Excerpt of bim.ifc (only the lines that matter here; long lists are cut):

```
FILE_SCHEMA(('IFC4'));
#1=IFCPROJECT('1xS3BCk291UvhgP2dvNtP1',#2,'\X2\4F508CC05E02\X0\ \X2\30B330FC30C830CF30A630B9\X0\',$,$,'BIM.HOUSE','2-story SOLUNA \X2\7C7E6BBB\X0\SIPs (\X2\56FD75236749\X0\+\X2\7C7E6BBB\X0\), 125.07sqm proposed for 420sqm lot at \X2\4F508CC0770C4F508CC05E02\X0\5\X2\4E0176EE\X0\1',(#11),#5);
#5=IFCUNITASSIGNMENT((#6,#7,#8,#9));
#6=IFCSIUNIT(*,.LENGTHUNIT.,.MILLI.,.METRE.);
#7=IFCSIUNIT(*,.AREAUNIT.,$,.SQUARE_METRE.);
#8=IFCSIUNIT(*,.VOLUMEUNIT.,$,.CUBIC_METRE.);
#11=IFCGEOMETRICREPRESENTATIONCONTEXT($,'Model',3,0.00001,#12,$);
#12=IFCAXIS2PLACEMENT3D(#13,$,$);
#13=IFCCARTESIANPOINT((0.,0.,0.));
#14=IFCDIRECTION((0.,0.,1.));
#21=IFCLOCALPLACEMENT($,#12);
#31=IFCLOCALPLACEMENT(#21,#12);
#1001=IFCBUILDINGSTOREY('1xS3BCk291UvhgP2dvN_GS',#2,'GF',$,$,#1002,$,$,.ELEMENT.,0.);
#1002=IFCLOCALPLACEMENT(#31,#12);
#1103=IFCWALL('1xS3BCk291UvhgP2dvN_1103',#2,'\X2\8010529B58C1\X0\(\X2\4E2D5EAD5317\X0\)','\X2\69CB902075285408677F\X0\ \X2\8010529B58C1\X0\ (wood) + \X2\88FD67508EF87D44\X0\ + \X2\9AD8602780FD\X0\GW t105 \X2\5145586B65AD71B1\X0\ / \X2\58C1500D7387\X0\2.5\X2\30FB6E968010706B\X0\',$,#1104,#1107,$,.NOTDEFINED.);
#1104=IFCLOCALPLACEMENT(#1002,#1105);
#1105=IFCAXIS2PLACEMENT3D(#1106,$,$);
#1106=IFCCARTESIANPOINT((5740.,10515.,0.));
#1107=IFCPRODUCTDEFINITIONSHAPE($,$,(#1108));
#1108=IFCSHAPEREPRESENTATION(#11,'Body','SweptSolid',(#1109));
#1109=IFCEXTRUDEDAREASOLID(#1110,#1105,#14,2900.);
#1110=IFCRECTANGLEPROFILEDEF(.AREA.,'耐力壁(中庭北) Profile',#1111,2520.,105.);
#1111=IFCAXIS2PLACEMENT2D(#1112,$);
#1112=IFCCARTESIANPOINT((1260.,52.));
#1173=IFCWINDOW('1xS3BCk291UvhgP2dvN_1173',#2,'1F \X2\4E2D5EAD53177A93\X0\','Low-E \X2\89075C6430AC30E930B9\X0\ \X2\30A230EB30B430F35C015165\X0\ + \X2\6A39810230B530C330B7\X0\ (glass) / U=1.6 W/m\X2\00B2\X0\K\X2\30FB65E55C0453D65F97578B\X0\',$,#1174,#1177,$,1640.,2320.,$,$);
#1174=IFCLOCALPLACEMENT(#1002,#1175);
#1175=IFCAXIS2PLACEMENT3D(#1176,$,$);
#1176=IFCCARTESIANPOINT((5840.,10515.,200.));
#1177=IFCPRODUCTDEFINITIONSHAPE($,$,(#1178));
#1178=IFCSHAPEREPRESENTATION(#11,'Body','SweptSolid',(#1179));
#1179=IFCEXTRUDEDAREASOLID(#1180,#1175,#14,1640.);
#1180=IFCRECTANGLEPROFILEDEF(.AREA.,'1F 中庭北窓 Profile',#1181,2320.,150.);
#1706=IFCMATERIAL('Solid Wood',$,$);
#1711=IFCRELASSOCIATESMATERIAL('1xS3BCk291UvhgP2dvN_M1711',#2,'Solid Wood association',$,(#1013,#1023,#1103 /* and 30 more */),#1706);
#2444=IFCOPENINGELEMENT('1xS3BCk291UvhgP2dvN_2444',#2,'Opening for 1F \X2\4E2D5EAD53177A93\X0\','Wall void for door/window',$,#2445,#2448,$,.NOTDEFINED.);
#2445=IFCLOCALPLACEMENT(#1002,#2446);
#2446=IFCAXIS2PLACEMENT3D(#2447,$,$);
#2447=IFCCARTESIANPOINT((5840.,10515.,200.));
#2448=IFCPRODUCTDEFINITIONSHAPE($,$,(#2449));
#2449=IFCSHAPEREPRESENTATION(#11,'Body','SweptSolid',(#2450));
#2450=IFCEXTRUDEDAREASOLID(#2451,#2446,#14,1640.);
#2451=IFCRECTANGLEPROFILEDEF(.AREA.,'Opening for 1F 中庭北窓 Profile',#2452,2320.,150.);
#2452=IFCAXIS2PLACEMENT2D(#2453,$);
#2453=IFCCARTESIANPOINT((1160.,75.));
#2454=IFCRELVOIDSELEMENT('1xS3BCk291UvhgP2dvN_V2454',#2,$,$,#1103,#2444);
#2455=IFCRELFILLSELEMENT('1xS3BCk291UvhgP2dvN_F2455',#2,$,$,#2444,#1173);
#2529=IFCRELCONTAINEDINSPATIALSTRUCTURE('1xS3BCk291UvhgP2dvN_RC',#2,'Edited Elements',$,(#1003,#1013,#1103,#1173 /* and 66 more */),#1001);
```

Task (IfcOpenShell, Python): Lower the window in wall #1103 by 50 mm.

```python
import numpy as np
import ifcopenshell
import ifcopenshell.api.geometry
import ifcopenshell.util.placement
import ifcopenshell.util.unit

model = ifcopenshell.open("bim.ifc")
unit_scale = ifcopenshell.util.unit.calculate_unit_scale(model)

window = model.by_id(1173)
opening = window.FillsVoids[0].RelatingOpeningElement
dz = -0.05 / unit_scale

shift = np.array([0.0, 0.0, dz])
# The window is not placed relative to its opening, so move both.
for product in (opening, window):
    matrix = ifcopenshell.util.placement.get_local_placement(product.ObjectPlacement)
    matrix[:3, 3] += shift
    ifcopenshell.api.geometry.edit_object_placement(model, product=product, matrix=matrix, is_si=False)

print(f"moved by {dz * unit_scale:+.3f} m")

model.write("bim_rev.ifc")
```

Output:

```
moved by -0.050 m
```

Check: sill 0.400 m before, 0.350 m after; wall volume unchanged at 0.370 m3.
